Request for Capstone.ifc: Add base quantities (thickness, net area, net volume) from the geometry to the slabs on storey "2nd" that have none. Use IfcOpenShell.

First a look at what the model holds.

```python
import ifcopenshell
import ifcopenshell.util.element
import ifcopenshell.util.unit

model = ifcopenshell.open("Capstone.ifc")
print(model.schema)
for unit_type in ("LENGTHUNIT", "AREAUNIT", "VOLUMEUNIT"):
    print(unit_type, ifcopenshell.util.unit.calculate_unit_scale(model, unit_type))
storey = next(s for s in model.by_type("IfcBuildingStorey") if s.Name == "2nd")
slabs = [e for e in ifcopenshell.util.element.get_decomposition(storey) if e.is_a("IfcSlab")]
for e in sorted(slabs, key=lambda e: e.id()):
    print(e.id(), e.is_a(), e.Name, list(ifcopenshell.util.element.get_psets(e, qtos_only=True)), sep=" | ")
```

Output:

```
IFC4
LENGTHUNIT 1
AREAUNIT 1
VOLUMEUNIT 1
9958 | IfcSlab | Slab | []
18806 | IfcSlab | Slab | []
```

```python
import ifcopenshell
import ifcopenshell.api.pset
import ifcopenshell.geom
import ifcopenshell.util.element
import ifcopenshell.util.shape
import ifcopenshell.util.unit

model = ifcopenshell.open("Capstone.ifc")
unit_scale = ifcopenshell.util.unit.calculate_unit_scale(model)
area_scale = ifcopenshell.util.unit.calculate_unit_scale(model, "AREAUNIT")
volume_scale = ifcopenshell.util.unit.calculate_unit_scale(model, "VOLUMEUNIT")
settings = ifcopenshell.geom.settings()

storey = next(s for s in model.by_type("IfcBuildingStorey") if s.Name == "2nd")
slabs = [e for e in ifcopenshell.util.element.get_decomposition(storey) if e.is_a("IfcSlab")]

for e in sorted(slabs, key=lambda e: e.id()):
    if ifcopenshell.util.element.get_psets(e, qtos_only=True, should_inherit=False):
        continue
    # Geometry comes back in metres, in the element's own axes.
    shape = ifcopenshell.geom.create_shape(settings, e)
    values = {
        "Width": ifcopenshell.util.shape.get_z(shape.geometry) / unit_scale,
        "NetArea": ifcopenshell.util.shape.get_footprint_area(shape.geometry) / area_scale,
        "NetVolume": ifcopenshell.util.shape.get_volume(shape.geometry) / volume_scale,
    }
    qto = ifcopenshell.api.pset.add_qto(model, product=e, name="Qto_SlabBaseQuantities")
    ifcopenshell.api.pset.edit_qto(model, qto=qto, properties=values)
    print(e.id(), {k: round(v, 3) for k, v in values.items()})

model.write("Capstone_rev.ifc")
```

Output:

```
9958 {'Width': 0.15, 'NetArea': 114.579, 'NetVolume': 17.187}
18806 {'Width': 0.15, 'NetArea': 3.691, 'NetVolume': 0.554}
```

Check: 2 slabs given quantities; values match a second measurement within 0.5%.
